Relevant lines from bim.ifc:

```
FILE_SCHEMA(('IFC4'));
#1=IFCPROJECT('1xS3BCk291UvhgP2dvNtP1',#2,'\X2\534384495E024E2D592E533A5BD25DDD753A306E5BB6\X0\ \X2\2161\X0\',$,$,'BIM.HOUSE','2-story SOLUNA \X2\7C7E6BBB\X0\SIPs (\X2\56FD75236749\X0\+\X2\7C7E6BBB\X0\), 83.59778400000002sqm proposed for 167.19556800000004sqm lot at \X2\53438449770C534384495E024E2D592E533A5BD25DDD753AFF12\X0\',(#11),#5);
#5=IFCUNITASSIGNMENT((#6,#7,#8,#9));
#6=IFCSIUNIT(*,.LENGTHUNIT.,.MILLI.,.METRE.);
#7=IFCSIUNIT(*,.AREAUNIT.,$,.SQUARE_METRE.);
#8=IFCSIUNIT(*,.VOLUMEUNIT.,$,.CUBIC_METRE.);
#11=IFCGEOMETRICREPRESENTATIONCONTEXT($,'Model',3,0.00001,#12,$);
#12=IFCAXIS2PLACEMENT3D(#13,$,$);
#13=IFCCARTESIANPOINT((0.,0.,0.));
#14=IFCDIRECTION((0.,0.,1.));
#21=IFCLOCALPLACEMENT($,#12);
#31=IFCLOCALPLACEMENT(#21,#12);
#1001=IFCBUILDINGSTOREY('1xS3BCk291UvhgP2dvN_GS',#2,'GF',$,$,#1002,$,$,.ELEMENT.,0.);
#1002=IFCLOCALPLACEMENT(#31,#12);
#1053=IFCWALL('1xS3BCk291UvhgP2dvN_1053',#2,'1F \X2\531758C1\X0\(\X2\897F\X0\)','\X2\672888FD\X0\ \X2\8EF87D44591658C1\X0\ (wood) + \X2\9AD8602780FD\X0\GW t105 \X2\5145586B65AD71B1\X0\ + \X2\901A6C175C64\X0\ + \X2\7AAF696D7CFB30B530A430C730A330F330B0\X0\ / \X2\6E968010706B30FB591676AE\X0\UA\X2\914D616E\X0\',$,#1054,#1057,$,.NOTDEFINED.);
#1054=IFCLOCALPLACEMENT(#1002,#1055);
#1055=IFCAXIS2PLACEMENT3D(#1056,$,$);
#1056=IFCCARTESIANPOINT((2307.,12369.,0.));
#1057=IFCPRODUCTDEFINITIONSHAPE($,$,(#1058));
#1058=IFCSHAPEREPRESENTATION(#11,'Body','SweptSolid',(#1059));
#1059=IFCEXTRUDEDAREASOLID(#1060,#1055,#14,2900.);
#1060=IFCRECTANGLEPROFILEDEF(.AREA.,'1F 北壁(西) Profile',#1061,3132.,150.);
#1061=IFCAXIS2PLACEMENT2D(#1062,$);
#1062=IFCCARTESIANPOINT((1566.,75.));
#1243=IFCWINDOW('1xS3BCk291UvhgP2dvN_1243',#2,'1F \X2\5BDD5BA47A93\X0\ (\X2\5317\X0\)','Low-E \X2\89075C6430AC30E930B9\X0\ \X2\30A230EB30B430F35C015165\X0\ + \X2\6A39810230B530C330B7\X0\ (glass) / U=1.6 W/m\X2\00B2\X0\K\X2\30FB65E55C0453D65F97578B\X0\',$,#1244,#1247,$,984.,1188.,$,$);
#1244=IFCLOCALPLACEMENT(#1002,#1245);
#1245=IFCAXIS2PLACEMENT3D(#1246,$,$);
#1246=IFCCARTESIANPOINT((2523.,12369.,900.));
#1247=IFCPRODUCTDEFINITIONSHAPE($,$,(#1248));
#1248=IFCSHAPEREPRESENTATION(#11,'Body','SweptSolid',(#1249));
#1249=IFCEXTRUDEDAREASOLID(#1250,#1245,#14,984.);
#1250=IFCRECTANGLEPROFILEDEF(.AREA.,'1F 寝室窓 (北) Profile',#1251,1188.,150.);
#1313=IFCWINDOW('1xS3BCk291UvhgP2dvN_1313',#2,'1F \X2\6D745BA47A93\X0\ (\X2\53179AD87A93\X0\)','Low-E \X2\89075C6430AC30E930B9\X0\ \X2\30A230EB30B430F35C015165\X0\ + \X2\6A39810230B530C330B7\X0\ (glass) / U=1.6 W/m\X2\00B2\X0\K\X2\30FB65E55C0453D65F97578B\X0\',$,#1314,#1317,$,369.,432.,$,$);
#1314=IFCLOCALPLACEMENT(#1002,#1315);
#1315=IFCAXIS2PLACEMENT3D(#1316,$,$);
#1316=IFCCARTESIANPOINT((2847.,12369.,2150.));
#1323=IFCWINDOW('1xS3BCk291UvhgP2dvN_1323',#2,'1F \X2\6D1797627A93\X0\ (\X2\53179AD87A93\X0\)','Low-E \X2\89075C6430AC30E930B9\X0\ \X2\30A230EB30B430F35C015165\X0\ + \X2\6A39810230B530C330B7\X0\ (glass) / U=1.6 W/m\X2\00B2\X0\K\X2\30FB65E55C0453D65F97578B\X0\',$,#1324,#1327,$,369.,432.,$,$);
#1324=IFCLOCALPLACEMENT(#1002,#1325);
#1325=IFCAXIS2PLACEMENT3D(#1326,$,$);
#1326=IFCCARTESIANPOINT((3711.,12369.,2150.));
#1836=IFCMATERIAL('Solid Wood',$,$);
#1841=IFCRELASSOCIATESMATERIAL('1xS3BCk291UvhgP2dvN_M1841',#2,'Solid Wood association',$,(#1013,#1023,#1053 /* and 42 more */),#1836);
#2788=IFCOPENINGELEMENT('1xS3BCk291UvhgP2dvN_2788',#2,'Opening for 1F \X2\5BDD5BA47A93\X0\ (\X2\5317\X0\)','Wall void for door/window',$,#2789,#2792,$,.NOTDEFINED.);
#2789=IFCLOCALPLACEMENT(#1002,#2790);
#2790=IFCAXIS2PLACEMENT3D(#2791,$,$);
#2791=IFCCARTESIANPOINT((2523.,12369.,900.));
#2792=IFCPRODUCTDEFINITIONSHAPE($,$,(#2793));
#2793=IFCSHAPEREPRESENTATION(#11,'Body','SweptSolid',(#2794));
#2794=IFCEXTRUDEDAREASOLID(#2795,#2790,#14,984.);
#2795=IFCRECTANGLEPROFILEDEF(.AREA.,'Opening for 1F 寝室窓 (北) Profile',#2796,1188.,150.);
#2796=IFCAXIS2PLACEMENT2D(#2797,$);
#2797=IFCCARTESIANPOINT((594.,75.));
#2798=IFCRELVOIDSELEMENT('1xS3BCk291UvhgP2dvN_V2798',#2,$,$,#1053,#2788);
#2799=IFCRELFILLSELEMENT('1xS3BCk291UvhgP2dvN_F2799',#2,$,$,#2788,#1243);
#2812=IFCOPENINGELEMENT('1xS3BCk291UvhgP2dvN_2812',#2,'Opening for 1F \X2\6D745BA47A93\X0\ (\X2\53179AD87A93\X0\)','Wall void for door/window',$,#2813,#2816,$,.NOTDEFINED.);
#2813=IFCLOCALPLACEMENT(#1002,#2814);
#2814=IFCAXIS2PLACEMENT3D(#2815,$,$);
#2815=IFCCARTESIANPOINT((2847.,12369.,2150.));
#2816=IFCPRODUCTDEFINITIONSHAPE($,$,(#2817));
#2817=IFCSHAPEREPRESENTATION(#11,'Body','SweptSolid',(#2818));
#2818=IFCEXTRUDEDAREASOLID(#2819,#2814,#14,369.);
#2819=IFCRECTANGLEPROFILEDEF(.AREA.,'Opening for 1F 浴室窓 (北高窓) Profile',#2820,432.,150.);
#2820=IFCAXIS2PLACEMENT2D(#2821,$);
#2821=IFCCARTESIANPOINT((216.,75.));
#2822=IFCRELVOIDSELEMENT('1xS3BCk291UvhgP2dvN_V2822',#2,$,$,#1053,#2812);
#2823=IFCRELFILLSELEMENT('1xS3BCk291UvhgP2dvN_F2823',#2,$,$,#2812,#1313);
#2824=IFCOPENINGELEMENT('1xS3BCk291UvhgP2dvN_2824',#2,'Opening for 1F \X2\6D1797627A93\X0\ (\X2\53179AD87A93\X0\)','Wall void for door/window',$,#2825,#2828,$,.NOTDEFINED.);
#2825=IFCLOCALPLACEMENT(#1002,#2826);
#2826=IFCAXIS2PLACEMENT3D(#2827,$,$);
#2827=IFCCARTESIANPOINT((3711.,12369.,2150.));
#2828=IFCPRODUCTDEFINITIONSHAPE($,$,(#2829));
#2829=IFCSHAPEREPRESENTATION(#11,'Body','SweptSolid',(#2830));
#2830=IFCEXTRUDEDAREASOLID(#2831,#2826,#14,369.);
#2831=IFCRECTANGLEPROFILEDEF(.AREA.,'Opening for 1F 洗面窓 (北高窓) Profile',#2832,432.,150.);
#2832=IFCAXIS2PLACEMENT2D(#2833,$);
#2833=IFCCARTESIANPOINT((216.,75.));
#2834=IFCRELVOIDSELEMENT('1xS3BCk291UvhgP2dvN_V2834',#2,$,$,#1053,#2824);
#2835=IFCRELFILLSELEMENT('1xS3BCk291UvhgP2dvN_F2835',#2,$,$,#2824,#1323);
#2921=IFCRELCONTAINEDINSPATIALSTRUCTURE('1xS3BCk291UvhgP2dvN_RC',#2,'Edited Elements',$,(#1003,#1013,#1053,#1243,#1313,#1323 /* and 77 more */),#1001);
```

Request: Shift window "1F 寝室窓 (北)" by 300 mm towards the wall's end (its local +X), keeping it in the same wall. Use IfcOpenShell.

```python
import ifcopenshell
import ifcopenshell.api.geometry
import ifcopenshell.util.placement
import ifcopenshell.util.unit

model = ifcopenshell.open("bim.ifc")
unit_scale = ifcopenshell.util.unit.calculate_unit_scale(model)

window = model.by_guid("1xS3BCk291UvhgP2dvN_1243")
opening = window.FillsVoids[0].RelatingOpeningElement
wall = opening.VoidsElements[0].RelatingBuildingElement

wall_matrix = ifcopenshell.util.placement.get_local_placement(wall.ObjectPlacement)
shift = wall_matrix[:3, 0] * 0.3 / unit_scale
before = ifcopenshell.util.placement.get_local_placement(window.ObjectPlacement)[:3, 3].copy()

# The window is not placed relative to its opening, so move both.
for product in (opening, window):
    matrix = ifcopenshell.util.placement.get_local_placement(product.ObjectPlacement)
    matrix[:3, 3] += shift
    ifcopenshell.api.geometry.edit_object_placement(model, product=product, matrix=matrix, is_si=False)

after = ifcopenshell.util.placement.get_local_placement(window.ObjectPlacement)[:3, 3]
print("window moved by", (after - before).round(3) + 0.0)

model.write("bim_updated.ifc")
```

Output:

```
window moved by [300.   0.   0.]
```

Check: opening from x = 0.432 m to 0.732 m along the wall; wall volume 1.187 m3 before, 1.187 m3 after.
